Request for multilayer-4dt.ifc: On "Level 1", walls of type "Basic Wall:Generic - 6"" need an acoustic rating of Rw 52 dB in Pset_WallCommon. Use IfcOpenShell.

First a look at what the model holds.

```python
import ifcopenshell
import ifcopenshell.util.element

model = ifcopenshell.open("multilayer-4dt.ifc")
print(model.schema)
storey = next(s for s in model.by_type("IfcBuildingStorey") if s.Name == "Level 1")
walls = [e for e in ifcopenshell.util.element.get_decomposition(storey) if e.is_a("IfcWall")]
seen = {}
for e in walls:
    element_type = ifcopenshell.util.element.get_type(e)
    key = (element_type.Name if element_type != e and element_type else None, ifcopenshell.util.element.get_pset(e, "Pset_WallCommon", "AcousticRating"))
    seen[key] = seen.get(key, 0) + 1
for (name, value), count in sorted(seen.items(), key=str):
    print(count, "x", name, "|", value)
```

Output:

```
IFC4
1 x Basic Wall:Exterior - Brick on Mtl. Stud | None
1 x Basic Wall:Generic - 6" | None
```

```python
import ifcopenshell
import ifcopenshell.api.pset
import ifcopenshell.util.element

model = ifcopenshell.open("multilayer-4dt.ifc")

storey = next(s for s in model.by_type("IfcBuildingStorey") if s.Name == "Level 1")
walls = [e for e in ifcopenshell.util.element.get_decomposition(storey) if e.is_a("IfcWall")]

count = 0
for e in walls:
    element_type = ifcopenshell.util.element.get_type(e)
    if element_type in (None, e) or element_type.Name != 'Basic Wall:Generic - 6"':
        continue
    # add_pset returns the element's existing set when there is one.
    pset = ifcopenshell.api.pset.add_pset(model, product=e, name="Pset_WallCommon")
    ifcopenshell.api.pset.edit_pset(model, pset=pset, properties={"AcousticRating": "Rw 52 dB"})
    count += 1

print(count, "walls updated")

model.write("multilayer-4dt_updated.ifc")
```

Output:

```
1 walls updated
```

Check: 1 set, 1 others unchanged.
